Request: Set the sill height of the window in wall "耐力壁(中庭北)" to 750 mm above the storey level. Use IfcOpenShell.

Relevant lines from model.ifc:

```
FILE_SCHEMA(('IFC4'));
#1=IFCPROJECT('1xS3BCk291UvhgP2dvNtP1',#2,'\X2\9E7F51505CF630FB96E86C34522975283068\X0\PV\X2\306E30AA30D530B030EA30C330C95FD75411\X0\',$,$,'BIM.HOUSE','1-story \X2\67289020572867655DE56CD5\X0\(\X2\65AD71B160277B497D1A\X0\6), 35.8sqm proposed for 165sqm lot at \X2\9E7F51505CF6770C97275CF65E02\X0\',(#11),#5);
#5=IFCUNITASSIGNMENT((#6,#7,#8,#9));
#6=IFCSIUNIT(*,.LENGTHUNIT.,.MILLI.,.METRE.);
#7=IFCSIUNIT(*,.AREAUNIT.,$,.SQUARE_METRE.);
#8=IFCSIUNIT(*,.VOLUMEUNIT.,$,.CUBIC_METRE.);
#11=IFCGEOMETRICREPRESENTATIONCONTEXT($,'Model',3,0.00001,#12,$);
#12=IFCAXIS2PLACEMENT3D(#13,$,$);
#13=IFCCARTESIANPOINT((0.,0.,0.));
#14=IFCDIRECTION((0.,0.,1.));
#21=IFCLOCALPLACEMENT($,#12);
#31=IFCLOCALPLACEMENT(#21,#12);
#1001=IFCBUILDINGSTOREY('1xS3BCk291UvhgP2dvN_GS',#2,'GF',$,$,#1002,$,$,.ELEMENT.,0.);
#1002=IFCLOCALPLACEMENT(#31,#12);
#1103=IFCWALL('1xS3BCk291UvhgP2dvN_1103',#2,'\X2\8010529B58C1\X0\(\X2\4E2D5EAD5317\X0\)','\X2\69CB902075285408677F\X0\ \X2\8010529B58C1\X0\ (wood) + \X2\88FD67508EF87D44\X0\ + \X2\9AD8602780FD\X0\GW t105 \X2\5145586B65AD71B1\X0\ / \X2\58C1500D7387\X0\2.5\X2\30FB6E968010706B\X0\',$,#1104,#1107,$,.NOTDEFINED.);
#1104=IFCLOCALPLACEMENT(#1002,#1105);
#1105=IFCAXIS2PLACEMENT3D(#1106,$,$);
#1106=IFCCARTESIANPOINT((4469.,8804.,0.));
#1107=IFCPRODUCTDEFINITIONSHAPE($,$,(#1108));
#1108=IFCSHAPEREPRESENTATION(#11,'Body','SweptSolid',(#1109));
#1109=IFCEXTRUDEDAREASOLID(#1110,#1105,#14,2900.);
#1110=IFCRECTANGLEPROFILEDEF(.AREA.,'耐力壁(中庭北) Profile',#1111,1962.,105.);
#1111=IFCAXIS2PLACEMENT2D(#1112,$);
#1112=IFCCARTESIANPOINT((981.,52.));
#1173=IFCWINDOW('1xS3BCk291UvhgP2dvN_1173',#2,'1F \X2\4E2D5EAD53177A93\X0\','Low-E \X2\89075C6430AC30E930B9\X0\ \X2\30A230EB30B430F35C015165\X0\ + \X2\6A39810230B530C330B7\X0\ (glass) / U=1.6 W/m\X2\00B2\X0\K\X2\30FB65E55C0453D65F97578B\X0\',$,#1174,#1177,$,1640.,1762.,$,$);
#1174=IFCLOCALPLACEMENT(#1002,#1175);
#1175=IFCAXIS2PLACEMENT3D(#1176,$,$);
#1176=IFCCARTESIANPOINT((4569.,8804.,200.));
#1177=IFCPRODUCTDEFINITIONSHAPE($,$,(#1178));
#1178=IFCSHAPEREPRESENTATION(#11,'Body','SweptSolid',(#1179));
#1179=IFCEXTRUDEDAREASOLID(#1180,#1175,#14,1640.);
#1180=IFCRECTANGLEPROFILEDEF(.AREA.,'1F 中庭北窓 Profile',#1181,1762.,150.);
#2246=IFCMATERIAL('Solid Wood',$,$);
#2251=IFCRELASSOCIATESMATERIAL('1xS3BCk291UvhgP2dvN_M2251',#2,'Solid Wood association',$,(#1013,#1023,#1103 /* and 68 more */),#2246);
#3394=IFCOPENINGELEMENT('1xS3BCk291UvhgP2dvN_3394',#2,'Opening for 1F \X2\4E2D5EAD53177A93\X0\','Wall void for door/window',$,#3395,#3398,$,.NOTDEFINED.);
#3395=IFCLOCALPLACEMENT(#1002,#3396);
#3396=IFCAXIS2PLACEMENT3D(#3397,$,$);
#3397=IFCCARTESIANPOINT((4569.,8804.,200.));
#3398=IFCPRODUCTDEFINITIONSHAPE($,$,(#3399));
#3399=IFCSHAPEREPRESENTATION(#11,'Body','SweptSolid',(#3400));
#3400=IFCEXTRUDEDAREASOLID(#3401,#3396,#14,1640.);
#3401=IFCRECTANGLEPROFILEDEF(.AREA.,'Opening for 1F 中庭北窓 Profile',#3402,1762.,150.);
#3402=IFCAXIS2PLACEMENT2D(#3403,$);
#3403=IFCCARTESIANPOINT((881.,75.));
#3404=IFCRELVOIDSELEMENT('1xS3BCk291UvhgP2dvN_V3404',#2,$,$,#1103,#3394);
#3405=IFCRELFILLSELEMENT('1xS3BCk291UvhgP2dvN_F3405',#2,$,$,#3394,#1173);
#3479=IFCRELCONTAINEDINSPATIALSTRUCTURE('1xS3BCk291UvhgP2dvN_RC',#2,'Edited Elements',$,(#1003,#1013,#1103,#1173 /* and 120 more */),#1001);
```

```python
import numpy as np
import ifcopenshell
import ifcopenshell.api.geometry
import ifcopenshell.geom
import ifcopenshell.util.element
import ifcopenshell.util.placement
import ifcopenshell.util.shape
import ifcopenshell.util.unit

model = ifcopenshell.open("model.ifc")
unit_scale = ifcopenshell.util.unit.calculate_unit_scale(model)

window = model.by_id(1173)
opening = window.FillsVoids[0].RelatingOpeningElement
storey = ifcopenshell.util.element.get_container(window, ifc_class="IfcBuildingStorey")
level = ifcopenshell.util.placement.get_local_placement(storey.ObjectPlacement)[2, 3]

# The opening's origin need not be at the sill, so measure its lowest point.
shape = ifcopenshell.geom.create_shape(ifcopenshell.geom.settings(), opening)
bottom = ifcopenshell.util.shape.get_shape_bottom_elevation(shape, shape.geometry) / unit_scale
dz = level + 0.75 / unit_scale - bottom

shift = np.array([0.0, 0.0, dz])
# The window is not placed relative to its opening, so move both.
for product in (opening, window):
    matrix = ifcopenshell.util.placement.get_local_placement(product.ObjectPlacement)
    matrix[:3, 3] += shift
    ifcopenshell.api.geometry.edit_object_placement(model, product=product, matrix=matrix, is_si=False)

print(f"moved by {dz * unit_scale:+.3f} m")

model.write("model_updated.ifc")
```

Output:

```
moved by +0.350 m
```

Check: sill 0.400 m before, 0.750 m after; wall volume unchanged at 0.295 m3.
